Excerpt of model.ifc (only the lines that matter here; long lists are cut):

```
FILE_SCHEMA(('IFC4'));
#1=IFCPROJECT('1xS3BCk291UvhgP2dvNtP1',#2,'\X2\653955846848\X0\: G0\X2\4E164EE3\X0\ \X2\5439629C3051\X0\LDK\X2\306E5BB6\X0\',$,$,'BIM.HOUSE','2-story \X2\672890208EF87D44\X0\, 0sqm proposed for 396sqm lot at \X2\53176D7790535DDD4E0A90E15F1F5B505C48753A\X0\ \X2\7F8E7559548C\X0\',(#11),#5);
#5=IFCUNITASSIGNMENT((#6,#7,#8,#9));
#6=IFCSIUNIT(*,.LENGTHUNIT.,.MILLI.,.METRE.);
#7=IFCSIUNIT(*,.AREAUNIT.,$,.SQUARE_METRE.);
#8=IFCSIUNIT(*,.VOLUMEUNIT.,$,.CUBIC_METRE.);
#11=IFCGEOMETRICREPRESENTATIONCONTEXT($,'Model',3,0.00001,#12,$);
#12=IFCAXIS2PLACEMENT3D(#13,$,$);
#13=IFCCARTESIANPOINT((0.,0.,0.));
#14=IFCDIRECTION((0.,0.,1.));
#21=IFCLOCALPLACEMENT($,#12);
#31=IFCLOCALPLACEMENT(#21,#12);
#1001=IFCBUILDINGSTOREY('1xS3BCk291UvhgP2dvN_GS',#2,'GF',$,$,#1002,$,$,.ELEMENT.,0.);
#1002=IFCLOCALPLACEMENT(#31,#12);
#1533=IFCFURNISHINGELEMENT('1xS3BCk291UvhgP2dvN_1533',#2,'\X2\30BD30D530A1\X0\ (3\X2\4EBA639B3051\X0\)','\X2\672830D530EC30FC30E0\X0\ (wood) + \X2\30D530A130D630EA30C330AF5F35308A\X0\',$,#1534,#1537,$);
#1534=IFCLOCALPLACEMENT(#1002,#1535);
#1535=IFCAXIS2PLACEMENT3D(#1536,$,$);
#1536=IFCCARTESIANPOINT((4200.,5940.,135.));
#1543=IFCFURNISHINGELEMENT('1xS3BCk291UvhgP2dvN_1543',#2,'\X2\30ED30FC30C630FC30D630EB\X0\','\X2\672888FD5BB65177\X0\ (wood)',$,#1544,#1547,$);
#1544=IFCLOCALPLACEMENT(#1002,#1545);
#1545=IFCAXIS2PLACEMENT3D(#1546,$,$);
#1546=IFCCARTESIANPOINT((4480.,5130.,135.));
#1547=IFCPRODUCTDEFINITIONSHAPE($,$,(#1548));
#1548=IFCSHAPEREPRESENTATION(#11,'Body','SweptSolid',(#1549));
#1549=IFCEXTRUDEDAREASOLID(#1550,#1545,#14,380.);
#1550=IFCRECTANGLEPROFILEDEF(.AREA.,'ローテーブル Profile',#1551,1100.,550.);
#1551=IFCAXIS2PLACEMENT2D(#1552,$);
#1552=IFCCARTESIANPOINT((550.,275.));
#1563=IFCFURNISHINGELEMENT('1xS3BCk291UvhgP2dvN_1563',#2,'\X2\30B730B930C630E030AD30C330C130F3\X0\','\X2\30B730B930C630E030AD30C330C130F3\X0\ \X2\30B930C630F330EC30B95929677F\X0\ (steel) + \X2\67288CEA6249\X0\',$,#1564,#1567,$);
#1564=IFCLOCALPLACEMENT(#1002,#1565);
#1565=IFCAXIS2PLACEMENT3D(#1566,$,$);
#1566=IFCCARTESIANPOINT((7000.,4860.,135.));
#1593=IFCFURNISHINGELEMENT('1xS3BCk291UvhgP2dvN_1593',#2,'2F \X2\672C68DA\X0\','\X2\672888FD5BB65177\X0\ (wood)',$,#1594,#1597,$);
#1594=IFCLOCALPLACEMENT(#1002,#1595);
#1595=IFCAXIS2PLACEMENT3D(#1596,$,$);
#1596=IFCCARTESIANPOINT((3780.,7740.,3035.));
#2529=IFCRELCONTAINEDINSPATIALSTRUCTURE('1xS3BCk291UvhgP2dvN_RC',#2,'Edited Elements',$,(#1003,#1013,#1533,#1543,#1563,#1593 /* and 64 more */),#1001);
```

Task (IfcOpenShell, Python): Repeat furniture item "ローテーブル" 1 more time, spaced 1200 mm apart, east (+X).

```python
import numpy as np
import ifcopenshell
import ifcopenshell.api.geometry
import ifcopenshell.api.root
import ifcopenshell.util.element
import ifcopenshell.util.placement

model = ifcopenshell.open("model.ifc")


def reuse_history(source, copy):
    """copy_class also copies each property set's owner history, people and application; keep the originals."""
    for rel in copy.IsDefinedBy:
        if rel.is_a("IfcRelDefinesByProperties") and (history := rel.RelatingPropertyDefinition.OwnerHistory):
            rel.RelatingPropertyDefinition.OwnerHistory = source.OwnerHistory
            ifcopenshell.util.element.remove_deep2(model, history)


source = model.by_id(1543)
base = ifcopenshell.util.placement.get_local_placement(source.ObjectPlacement)
step = np.array([1.0, 0.0, 0.0]) * 1200.0

for i in range(1, 2):
    copy = ifcopenshell.api.root.copy_class(model, product=source)
    copy.Representation = ifcopenshell.util.element.copy_deep(
        model, source.Representation, exclude=["IfcGeometricRepresentationContext", "IfcRepresentationMap"]
    )
    reuse_history(source, copy)
    matrix = base.copy()
    matrix[:3, 3] += i * step
    print("added at", matrix[:3, 3].round(3) + 0.0)
    ifcopenshell.api.geometry.edit_object_placement(model, product=copy, matrix=matrix, is_si=False)

model.write("model_edited.ifc")
```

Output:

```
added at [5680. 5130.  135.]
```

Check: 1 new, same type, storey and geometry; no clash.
